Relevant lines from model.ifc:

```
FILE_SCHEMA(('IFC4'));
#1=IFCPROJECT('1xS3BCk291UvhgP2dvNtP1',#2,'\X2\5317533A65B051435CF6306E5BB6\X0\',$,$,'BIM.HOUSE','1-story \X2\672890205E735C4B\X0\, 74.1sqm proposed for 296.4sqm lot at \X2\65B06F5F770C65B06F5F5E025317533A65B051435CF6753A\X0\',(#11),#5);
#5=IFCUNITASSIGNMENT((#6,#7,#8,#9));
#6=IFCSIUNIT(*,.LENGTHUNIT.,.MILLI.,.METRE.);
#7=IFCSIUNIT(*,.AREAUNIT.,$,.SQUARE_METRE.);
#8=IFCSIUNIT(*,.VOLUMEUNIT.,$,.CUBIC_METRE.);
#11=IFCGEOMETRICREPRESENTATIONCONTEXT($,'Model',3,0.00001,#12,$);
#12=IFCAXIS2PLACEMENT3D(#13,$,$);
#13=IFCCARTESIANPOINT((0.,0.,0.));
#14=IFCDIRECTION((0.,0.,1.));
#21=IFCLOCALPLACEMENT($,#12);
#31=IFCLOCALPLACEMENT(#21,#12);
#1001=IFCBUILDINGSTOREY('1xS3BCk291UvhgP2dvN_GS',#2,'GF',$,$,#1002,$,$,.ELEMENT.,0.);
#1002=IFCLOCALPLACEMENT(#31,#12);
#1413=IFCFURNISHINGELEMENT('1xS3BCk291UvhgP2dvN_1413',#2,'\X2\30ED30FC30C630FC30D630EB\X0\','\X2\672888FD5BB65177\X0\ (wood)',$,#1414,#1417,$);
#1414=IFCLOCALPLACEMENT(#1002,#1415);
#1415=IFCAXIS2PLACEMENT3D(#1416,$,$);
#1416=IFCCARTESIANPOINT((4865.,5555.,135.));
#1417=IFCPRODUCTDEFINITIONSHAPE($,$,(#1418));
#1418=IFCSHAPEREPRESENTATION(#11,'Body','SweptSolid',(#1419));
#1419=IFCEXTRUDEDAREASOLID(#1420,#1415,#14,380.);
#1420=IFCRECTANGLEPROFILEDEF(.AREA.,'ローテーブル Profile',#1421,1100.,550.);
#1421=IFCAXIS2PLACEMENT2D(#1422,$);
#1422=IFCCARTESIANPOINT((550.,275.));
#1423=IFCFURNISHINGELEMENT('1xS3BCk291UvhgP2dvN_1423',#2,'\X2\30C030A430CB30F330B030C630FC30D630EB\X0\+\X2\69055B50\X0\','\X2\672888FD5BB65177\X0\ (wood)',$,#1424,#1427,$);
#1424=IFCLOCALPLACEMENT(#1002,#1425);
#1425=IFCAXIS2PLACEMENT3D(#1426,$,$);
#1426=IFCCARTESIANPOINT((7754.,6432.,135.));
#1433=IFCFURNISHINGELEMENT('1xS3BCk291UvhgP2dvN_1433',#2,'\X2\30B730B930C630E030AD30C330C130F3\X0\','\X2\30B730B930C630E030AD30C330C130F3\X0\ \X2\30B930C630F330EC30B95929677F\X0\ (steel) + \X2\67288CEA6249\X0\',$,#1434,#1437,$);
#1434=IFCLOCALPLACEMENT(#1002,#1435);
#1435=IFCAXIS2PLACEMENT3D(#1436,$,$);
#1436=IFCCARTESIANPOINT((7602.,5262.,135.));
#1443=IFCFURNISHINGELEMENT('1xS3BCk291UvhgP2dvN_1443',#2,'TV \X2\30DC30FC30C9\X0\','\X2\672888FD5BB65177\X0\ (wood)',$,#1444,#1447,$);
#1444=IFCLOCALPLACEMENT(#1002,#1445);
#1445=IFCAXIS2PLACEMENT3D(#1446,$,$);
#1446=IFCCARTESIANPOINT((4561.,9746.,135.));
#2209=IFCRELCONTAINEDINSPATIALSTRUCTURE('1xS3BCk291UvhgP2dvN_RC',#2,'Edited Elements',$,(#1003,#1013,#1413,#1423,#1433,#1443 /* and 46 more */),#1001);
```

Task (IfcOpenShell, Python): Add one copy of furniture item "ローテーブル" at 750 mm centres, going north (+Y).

```python
import numpy as np
import ifcopenshell
import ifcopenshell.api.geometry
import ifcopenshell.api.root
import ifcopenshell.util.element
import ifcopenshell.util.placement
import ifcopenshell.util.unit

model = ifcopenshell.open("model.ifc")
unit_scale = ifcopenshell.util.unit.calculate_unit_scale(model)


def reuse_history(source, copy):
    """copy_class also copies each property set's owner history, people and application; keep the originals."""
    for rel in copy.IsDefinedBy:
        if rel.is_a("IfcRelDefinesByProperties") and (history := rel.RelatingPropertyDefinition.OwnerHistory):
            rel.RelatingPropertyDefinition.OwnerHistory = source.OwnerHistory
            ifcopenshell.util.element.remove_deep2(model, history)


source = model.by_id(1413)
base = ifcopenshell.util.placement.get_local_placement(source.ObjectPlacement)
step = np.array([0.0, 1.0, 0.0]) * 0.75 / unit_scale

for i in range(1, 2):
    copy = ifcopenshell.api.root.copy_class(model, product=source)
    copy.Representation = ifcopenshell.util.element.copy_deep(
        model, source.Representation, exclude=["IfcGeometricRepresentationContext", "IfcRepresentationMap"]
    )
    reuse_history(source, copy)
    matrix = base.copy()
    matrix[:3, 3] += i * step
    print("added at", matrix[:3, 3].round(3) + 0.0)
    ifcopenshell.api.geometry.edit_object_placement(model, product=copy, matrix=matrix, is_si=False)

model.write("model_edited.ifc")
```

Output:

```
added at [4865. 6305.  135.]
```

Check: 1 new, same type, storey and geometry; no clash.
